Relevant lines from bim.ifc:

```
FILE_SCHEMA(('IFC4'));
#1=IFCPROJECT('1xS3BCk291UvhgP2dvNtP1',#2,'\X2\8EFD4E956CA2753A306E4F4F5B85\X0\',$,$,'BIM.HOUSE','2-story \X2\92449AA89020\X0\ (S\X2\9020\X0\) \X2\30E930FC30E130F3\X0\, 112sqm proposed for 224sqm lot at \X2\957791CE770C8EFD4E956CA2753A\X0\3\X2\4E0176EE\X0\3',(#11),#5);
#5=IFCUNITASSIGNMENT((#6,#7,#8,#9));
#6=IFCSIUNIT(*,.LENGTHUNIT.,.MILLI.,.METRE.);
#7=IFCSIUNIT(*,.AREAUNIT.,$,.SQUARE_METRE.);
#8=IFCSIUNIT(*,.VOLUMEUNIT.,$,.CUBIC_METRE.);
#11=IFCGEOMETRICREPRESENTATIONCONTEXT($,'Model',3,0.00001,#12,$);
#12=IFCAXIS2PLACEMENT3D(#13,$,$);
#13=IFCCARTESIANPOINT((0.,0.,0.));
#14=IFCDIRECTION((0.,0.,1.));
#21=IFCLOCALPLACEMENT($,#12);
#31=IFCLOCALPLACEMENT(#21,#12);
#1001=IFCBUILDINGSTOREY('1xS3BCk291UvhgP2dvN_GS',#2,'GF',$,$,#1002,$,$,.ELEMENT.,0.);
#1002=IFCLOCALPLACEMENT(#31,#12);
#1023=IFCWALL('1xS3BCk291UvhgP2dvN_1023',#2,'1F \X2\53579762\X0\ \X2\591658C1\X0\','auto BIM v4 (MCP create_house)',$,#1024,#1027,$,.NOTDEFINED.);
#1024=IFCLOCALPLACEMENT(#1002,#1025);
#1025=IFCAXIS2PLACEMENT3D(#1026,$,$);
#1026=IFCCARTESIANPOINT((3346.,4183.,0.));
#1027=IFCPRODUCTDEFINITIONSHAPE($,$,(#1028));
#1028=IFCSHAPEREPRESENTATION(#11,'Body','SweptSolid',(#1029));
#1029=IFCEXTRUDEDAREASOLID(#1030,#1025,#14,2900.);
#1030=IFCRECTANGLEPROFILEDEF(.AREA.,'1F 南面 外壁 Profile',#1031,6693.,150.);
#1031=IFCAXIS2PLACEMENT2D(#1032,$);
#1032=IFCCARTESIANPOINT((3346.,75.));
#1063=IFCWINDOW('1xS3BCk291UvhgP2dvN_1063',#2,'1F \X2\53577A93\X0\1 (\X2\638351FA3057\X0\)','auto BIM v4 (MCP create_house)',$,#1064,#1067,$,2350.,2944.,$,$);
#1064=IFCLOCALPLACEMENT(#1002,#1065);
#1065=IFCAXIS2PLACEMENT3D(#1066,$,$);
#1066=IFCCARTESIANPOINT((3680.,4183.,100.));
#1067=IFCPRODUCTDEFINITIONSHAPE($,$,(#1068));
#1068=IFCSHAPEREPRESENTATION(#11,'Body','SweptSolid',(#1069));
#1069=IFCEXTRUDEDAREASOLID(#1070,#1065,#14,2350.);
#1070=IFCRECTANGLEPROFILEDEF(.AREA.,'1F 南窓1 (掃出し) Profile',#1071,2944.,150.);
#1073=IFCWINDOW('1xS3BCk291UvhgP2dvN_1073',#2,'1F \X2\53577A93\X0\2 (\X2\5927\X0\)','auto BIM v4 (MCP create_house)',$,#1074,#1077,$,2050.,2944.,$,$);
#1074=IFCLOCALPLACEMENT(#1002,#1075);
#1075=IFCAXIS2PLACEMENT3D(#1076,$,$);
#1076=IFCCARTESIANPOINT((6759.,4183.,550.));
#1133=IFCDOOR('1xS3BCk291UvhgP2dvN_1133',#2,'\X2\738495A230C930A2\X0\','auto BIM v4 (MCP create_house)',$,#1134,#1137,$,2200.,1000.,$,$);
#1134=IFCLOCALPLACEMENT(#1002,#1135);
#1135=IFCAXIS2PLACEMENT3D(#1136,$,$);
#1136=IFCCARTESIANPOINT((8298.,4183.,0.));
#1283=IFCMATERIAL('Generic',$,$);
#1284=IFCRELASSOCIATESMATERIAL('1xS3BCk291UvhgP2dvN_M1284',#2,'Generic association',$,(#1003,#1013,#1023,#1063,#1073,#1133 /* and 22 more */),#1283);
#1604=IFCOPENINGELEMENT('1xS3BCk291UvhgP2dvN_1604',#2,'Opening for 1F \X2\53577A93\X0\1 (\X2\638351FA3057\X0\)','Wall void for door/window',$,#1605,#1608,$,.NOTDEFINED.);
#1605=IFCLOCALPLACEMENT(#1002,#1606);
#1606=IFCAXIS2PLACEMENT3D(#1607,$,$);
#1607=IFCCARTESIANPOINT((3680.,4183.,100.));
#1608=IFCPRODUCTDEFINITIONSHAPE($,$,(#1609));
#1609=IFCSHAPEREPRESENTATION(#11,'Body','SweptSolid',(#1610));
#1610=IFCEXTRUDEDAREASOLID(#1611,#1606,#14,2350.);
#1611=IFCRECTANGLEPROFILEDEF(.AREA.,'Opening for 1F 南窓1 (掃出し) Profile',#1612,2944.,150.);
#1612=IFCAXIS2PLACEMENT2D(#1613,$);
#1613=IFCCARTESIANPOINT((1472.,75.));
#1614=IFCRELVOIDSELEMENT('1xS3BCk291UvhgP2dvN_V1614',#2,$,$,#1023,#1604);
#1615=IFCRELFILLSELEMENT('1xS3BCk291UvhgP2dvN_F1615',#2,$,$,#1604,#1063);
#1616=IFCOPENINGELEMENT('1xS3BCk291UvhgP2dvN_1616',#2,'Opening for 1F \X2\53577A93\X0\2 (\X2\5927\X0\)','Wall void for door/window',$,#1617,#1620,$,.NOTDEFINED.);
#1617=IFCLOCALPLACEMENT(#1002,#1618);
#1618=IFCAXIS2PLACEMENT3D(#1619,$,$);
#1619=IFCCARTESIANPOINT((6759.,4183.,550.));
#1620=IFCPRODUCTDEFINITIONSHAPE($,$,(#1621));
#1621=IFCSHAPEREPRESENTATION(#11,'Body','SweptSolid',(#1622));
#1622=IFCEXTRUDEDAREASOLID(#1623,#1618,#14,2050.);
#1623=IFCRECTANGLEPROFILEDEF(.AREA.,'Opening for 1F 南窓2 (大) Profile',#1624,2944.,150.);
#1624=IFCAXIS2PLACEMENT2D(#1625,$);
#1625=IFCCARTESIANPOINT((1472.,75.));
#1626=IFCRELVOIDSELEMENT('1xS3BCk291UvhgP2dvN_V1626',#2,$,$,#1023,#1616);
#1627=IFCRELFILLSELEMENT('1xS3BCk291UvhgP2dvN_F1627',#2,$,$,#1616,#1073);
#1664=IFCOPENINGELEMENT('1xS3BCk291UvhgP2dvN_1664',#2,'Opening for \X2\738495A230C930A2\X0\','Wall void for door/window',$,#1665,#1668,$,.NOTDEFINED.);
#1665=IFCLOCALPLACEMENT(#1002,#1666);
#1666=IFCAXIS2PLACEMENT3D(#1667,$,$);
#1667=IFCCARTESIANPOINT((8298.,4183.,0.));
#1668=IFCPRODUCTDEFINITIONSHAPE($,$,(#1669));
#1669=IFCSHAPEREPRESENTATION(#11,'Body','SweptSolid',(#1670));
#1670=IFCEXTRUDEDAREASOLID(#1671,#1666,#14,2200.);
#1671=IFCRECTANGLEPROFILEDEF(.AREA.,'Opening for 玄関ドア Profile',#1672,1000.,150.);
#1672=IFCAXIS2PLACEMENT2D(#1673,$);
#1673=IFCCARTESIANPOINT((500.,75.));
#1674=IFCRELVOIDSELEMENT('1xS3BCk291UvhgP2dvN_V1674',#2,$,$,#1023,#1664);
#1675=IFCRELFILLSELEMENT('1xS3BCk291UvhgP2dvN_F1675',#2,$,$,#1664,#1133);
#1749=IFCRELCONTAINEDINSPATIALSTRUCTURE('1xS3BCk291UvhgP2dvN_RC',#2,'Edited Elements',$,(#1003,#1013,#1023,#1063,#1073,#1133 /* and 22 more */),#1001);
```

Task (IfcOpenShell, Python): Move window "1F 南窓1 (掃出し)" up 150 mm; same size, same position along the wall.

```python
import numpy as np
import ifcopenshell
import ifcopenshell.api.geometry
import ifcopenshell.util.placement
import ifcopenshell.util.unit

model = ifcopenshell.open("bim.ifc")
unit_scale = ifcopenshell.util.unit.calculate_unit_scale(model)

window = model.by_guid("1xS3BCk291UvhgP2dvN_1063")
opening = window.FillsVoids[0].RelatingOpeningElement
dz = 150.0

shift = np.array([0.0, 0.0, dz])
# The window is not placed relative to its opening, so move both.
for product in (opening, window):
    matrix = ifcopenshell.util.placement.get_local_placement(product.ObjectPlacement)
    matrix[:3, 3] += shift
    ifcopenshell.api.geometry.edit_object_placement(model, product=product, matrix=matrix, is_si=False)

print(f"moved by {dz * unit_scale:+.3f} m")

model.write("bim_edited.ifc")
```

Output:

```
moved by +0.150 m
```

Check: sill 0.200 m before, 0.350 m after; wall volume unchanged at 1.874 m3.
